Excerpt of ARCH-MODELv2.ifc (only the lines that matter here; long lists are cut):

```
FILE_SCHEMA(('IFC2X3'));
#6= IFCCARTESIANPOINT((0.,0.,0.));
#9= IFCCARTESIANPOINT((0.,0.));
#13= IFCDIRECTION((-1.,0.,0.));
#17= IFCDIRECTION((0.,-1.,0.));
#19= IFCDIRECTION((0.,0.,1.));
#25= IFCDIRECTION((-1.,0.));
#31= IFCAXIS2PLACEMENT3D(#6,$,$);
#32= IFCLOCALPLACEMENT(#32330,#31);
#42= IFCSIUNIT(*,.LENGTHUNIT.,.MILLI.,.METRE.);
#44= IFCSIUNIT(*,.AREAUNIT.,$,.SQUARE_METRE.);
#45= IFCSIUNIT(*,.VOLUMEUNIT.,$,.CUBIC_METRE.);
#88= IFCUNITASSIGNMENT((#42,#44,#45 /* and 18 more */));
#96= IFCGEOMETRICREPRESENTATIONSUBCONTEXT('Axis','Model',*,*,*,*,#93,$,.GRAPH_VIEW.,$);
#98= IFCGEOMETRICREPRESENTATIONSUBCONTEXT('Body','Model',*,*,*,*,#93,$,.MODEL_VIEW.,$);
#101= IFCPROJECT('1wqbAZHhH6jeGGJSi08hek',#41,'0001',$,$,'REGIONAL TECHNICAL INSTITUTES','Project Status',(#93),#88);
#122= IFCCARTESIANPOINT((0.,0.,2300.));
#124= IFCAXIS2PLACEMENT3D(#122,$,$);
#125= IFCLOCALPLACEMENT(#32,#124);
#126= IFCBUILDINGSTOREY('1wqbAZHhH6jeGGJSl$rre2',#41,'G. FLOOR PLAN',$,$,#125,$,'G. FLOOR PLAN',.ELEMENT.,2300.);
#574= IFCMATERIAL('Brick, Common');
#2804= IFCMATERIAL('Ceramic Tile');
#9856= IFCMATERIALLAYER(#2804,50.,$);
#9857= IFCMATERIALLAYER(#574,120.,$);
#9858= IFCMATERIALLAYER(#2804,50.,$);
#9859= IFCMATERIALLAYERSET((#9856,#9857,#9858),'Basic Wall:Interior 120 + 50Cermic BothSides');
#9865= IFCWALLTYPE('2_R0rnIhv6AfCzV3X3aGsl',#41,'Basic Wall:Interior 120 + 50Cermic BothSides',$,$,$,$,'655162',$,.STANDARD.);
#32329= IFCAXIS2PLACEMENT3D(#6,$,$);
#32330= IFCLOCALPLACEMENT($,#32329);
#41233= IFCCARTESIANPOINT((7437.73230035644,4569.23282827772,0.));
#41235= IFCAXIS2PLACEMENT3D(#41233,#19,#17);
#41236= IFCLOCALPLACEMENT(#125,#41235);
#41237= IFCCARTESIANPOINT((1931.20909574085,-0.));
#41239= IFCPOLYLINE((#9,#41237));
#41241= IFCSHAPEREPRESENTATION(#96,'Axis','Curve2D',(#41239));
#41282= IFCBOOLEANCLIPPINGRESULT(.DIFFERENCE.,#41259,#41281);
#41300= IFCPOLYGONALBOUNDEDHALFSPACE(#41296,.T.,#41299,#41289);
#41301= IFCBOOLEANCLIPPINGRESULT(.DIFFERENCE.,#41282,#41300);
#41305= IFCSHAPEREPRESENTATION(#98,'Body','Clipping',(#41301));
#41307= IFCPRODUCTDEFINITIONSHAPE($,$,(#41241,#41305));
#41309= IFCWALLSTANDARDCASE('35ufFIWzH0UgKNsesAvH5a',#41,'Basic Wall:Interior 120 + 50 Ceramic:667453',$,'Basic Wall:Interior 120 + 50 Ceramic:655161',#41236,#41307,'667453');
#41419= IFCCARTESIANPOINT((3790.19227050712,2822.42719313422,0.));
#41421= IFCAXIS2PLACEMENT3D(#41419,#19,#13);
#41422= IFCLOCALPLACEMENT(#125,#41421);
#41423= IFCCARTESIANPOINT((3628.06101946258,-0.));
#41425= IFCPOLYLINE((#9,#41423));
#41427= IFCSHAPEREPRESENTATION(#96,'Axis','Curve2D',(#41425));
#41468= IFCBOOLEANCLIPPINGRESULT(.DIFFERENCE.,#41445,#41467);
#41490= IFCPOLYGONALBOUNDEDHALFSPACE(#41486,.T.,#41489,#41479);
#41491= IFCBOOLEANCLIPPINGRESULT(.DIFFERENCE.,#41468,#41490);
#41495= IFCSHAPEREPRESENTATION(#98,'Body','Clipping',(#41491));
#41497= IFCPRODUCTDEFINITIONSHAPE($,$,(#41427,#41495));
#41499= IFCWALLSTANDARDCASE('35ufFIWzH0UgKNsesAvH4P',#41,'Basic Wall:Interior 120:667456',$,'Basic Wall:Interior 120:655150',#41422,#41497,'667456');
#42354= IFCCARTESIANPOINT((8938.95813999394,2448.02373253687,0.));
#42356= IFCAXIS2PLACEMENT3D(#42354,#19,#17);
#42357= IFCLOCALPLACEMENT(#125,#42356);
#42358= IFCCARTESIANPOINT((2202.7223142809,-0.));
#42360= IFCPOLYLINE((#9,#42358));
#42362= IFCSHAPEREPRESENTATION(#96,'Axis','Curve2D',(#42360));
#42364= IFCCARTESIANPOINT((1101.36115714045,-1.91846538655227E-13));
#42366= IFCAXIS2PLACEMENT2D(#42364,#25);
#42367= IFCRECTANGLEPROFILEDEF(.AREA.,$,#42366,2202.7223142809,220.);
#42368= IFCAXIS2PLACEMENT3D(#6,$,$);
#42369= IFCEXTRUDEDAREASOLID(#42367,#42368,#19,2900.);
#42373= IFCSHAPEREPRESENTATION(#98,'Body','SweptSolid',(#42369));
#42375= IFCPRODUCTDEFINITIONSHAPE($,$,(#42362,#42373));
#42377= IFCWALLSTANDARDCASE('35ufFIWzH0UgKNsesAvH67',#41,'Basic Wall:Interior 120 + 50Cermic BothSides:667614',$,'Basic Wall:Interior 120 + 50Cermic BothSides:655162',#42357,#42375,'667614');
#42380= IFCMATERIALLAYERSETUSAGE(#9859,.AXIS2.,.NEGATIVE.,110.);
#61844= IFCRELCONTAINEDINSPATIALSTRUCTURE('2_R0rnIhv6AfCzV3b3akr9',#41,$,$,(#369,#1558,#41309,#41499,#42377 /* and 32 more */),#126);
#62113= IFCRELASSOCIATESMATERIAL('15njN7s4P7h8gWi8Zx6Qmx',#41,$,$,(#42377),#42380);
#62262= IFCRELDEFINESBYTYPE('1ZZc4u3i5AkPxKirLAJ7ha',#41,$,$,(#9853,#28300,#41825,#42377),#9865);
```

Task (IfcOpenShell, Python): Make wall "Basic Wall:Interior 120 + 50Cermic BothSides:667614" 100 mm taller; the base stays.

```python
import ifcopenshell
import ifcopenshell.geom
import ifcopenshell.util.representation
import ifcopenshell.util.shape

model = ifcopenshell.open("ARCH-MODELv2.ifc")
settings = ifcopenshell.geom.settings()


def volume(element):
    """Net volume in cubic metres, openings subtracted."""
    shape = ifcopenshell.geom.create_shape(settings, element)
    return ifcopenshell.util.shape.get_volume(shape.geometry)


wall = model.by_id(42377)
before = volume(wall)

body = ifcopenshell.util.representation.get_representation(wall, "Model", "Body")
solid = body.Items[0]
old_height = solid.Depth
solid.Depth += 100.0
after = volume(wall)

print(f"height {old_height:g} -> {solid.Depth:g}, volume {before:.3f} -> {after:.3f} m3")

model.write("ARCH-MODELv2_rev.ifc")
```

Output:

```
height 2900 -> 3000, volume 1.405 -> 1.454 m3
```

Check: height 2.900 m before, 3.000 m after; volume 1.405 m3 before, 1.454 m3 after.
